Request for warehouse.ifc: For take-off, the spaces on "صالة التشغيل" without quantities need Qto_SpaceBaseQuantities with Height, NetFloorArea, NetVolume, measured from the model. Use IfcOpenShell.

First a look at what the model holds.

```python
import ifcopenshell
import ifcopenshell.util.element
import ifcopenshell.util.unit

model = ifcopenshell.open("warehouse.ifc")
print(model.schema)
for unit_type in ("LENGTHUNIT", "AREAUNIT", "VOLUMEUNIT"):
    print(unit_type, ifcopenshell.util.unit.calculate_unit_scale(model, unit_type))
storey = next(s for s in model.by_type("IfcBuildingStorey") if s.Name == "صالة التشغيل")
spaces = [e for e in ifcopenshell.util.element.get_decomposition(storey) if e.is_a("IfcSpace")]
for e in sorted(spaces, key=lambda e: e.id()):
    print(e.id(), e.is_a(), e.Name, list(ifcopenshell.util.element.get_psets(e, qtos_only=True)), sep=" | ")
```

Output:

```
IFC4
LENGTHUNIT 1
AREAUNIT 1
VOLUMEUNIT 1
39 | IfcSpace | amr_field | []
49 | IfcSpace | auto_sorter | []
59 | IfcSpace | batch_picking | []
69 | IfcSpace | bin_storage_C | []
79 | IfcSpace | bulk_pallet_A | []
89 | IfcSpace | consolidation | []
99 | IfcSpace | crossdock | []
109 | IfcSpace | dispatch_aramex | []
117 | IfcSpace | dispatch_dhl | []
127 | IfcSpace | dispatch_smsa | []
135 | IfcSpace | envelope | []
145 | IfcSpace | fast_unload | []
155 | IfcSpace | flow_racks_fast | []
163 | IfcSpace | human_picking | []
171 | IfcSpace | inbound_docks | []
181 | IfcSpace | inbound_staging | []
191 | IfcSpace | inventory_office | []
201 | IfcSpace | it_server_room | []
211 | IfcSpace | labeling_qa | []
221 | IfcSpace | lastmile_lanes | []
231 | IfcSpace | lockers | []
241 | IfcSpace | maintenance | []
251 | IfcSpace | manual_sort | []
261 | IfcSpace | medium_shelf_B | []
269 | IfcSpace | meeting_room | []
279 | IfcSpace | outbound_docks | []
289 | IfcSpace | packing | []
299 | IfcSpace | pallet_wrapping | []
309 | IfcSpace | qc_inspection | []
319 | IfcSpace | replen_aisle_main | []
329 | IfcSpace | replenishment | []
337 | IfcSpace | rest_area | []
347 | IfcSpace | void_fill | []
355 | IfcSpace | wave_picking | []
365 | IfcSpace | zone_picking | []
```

```python
import ifcopenshell
import ifcopenshell.api.pset
import ifcopenshell.geom
import ifcopenshell.util.element
import ifcopenshell.util.shape
import ifcopenshell.util.unit

model = ifcopenshell.open("warehouse.ifc")
unit_scale = ifcopenshell.util.unit.calculate_unit_scale(model)
area_scale = ifcopenshell.util.unit.calculate_unit_scale(model, "AREAUNIT")
volume_scale = ifcopenshell.util.unit.calculate_unit_scale(model, "VOLUMEUNIT")
settings = ifcopenshell.geom.settings()

storey = next(s for s in model.by_type("IfcBuildingStorey") if s.Name == "صالة التشغيل")
spaces = [e for e in ifcopenshell.util.element.get_decomposition(storey) if e.is_a("IfcSpace")]

for e in sorted(spaces, key=lambda e: e.id()):
    if ifcopenshell.util.element.get_psets(e, qtos_only=True, should_inherit=False):
        continue
    # Geometry comes back in metres, in the element's own axes.
    shape = ifcopenshell.geom.create_shape(settings, e)
    values = {
        "Height": ifcopenshell.util.shape.get_z(shape.geometry) / unit_scale,
        "NetFloorArea": ifcopenshell.util.shape.get_footprint_area(shape.geometry) / area_scale,
        "NetVolume": ifcopenshell.util.shape.get_volume(shape.geometry) / volume_scale,
    }
    qto = ifcopenshell.api.pset.add_qto(model, product=e, name="Qto_SpaceBaseQuantities")
    ifcopenshell.api.pset.edit_qto(model, qto=qto, properties=values)
    print(e.id(), {k: round(v, 3) for k, v in values.items()})

model.write("warehouse_edited.ifc")
```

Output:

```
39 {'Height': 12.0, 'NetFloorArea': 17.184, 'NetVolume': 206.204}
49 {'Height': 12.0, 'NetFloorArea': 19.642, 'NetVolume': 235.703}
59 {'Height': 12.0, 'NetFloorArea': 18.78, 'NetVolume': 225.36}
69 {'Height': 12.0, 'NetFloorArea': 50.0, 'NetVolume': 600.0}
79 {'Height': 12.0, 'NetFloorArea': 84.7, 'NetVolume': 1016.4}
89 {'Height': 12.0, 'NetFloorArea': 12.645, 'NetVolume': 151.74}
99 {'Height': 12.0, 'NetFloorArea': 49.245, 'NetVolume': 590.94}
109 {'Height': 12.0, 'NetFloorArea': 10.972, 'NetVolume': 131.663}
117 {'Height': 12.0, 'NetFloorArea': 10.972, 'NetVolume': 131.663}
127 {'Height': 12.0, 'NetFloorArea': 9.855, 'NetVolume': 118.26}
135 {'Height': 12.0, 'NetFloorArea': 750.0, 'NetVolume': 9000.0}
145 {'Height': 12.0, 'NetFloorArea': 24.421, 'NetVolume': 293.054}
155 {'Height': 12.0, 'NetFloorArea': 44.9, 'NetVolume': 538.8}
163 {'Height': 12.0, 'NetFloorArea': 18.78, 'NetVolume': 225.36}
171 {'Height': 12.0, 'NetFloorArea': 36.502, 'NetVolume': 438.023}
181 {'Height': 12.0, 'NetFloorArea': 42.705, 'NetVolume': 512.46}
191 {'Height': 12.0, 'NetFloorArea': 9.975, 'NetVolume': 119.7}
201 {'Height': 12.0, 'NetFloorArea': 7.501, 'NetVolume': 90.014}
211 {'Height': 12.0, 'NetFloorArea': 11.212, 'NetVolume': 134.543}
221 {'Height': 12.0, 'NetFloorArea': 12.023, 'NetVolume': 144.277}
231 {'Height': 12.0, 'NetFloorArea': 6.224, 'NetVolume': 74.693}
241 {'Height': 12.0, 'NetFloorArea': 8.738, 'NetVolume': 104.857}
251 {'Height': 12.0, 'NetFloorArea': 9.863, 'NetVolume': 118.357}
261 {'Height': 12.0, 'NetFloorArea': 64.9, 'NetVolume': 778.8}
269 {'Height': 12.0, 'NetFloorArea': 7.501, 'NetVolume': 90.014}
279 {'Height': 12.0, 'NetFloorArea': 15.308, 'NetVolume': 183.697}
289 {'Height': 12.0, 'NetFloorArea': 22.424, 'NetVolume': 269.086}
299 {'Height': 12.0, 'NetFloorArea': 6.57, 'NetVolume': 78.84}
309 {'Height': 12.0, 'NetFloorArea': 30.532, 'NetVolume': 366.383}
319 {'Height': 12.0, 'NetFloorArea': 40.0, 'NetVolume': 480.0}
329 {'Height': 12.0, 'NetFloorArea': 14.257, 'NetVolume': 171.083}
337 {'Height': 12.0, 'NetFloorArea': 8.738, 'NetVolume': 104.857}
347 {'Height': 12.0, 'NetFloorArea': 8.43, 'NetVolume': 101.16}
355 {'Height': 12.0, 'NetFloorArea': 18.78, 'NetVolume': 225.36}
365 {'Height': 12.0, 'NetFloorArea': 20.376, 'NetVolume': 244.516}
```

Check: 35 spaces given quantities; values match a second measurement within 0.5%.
